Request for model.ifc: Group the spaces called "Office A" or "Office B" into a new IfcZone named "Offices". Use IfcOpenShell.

First a look at what the model holds.

```python
import ifcopenshell

model = ifcopenshell.open("model.ifc")
print(model.schema)
seen = {}
for space in model.by_type("IfcSpace"):
    seen[space.LongName] = seen.get(space.LongName, 0) + 1
for name, count in sorted(seen.items(), key=str):
    print(count, "x", name)
print("zones:", [z.Name for z in model.by_type("IfcZone")][:20])
```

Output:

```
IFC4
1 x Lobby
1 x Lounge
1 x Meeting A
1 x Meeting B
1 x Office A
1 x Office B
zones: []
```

```python
import ifcopenshell
import ifcopenshell.api.group
import ifcopenshell.api.root

model = ifcopenshell.open("model.ifc")

names = {"Office A", "Office B"}
spaces = [s for s in model.by_type("IfcSpace") if s.LongName in names]

zone = ifcopenshell.api.root.create_entity(model, ifc_class="IfcZone", name="Offices")
ifcopenshell.api.group.assign_group(model, products=spaces, group=zone)
print(len(spaces), "spaces in", zone.Name)

model.write("model_edited.ifc")
```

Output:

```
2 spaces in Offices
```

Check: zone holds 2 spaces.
